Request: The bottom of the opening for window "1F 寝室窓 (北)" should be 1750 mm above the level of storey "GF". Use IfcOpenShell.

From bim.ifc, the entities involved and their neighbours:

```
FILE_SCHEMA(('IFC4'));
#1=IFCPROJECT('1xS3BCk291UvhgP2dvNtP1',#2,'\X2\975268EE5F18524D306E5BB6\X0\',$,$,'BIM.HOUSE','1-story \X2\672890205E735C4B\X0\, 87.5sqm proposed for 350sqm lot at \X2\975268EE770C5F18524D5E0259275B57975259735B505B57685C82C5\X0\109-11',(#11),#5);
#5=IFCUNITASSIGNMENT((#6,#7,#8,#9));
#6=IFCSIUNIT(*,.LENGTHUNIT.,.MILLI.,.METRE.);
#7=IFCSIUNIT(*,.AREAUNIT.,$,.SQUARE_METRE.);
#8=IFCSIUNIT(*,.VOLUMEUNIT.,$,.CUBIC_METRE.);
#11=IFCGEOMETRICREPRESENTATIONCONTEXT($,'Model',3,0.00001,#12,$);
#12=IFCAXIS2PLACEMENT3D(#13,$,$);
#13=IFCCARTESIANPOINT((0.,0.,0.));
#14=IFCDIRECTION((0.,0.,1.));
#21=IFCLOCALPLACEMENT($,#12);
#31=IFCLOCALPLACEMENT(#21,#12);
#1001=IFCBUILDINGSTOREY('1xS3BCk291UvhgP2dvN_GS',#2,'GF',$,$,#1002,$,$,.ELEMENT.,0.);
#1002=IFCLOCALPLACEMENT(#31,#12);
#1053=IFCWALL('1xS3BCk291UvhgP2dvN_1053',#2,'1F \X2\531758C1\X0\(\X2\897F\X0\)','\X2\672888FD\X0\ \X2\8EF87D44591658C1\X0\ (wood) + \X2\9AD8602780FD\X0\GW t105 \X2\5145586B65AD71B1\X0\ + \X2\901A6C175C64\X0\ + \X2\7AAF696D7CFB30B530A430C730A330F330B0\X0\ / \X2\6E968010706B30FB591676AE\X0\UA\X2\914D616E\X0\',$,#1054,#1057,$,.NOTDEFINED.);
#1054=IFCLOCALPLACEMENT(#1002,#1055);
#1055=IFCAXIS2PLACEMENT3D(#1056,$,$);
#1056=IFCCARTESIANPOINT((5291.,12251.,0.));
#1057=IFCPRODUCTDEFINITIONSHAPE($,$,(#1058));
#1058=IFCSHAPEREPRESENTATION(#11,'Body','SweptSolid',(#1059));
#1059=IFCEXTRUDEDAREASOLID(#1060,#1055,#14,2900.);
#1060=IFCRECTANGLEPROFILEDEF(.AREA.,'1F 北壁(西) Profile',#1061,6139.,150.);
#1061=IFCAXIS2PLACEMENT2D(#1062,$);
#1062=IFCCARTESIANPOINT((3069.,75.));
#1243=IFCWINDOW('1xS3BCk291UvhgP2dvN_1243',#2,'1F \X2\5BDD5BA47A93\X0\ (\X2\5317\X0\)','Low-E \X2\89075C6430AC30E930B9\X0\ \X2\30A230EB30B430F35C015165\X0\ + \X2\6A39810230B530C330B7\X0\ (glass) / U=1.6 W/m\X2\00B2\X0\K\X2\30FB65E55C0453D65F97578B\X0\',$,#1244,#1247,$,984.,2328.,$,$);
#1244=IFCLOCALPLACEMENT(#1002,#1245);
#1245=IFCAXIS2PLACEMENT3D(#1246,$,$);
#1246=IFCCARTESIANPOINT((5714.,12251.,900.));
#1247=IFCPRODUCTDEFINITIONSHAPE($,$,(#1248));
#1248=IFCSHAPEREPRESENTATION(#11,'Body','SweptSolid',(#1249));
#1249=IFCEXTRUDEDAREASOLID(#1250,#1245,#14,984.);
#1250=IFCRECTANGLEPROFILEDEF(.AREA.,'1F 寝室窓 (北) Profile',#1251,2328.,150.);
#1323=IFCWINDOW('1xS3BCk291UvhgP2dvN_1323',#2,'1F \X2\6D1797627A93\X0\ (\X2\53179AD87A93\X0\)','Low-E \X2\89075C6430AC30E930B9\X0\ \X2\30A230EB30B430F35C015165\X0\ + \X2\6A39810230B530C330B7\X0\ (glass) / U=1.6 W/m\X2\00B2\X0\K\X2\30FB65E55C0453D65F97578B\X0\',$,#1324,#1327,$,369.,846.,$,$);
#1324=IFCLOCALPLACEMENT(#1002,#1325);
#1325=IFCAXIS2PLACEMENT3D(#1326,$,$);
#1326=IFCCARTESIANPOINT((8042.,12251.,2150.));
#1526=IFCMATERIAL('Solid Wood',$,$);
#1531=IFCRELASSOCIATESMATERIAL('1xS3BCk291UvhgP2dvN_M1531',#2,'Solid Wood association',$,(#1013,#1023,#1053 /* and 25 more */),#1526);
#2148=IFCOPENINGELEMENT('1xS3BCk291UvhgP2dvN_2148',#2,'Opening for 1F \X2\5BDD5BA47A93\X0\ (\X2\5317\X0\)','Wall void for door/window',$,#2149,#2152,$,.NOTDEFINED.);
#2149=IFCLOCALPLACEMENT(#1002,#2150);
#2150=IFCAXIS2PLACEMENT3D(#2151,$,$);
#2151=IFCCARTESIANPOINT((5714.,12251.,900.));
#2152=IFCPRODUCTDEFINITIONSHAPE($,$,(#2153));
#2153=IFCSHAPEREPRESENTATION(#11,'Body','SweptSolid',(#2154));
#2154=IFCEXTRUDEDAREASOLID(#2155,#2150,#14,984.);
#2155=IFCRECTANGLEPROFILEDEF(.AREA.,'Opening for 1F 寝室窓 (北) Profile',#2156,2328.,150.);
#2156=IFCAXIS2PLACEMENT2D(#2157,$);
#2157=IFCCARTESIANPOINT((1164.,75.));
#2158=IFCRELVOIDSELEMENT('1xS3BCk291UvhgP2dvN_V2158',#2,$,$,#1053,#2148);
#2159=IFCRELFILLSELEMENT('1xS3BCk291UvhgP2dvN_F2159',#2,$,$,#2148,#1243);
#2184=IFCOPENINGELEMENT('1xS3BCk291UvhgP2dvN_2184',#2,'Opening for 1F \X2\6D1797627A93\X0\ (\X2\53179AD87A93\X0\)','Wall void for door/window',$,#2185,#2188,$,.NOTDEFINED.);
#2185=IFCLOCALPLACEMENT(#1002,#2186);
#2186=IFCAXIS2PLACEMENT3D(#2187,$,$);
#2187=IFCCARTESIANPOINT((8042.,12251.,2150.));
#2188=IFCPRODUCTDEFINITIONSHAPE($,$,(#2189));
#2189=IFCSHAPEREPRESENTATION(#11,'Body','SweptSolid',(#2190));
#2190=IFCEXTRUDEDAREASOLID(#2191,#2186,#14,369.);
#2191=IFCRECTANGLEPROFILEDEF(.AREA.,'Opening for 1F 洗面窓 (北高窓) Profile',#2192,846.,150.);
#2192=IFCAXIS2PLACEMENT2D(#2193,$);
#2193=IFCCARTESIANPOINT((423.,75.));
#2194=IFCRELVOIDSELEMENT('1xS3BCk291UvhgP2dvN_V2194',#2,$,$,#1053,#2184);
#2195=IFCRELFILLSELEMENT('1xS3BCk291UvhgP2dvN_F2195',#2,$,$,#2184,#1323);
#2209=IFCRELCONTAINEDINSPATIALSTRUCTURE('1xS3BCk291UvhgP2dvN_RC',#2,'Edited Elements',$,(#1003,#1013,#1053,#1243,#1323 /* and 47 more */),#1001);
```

```python
import numpy as np
import ifcopenshell
import ifcopenshell.api.geometry
import ifcopenshell.geom
import ifcopenshell.util.element
import ifcopenshell.util.placement
import ifcopenshell.util.shape
import ifcopenshell.util.unit

model = ifcopenshell.open("bim.ifc")
unit_scale = ifcopenshell.util.unit.calculate_unit_scale(model)

window = model.by_id(1243)
opening = window.FillsVoids[0].RelatingOpeningElement
storey = ifcopenshell.util.element.get_container(window, ifc_class="IfcBuildingStorey")
level = ifcopenshell.util.placement.get_local_placement(storey.ObjectPlacement)[2, 3]

# The opening's origin need not be at the sill, so measure its lowest point.
shape = ifcopenshell.geom.create_shape(ifcopenshell.geom.settings(), opening)
bottom = ifcopenshell.util.shape.get_shape_bottom_elevation(shape, shape.geometry) / unit_scale
dz = level + 1750.0 - bottom

shift = np.array([0.0, 0.0, dz])
# The window is not placed relative to its opening, so move both.
for product in (opening, window):
    matrix = ifcopenshell.util.placement.get_local_placement(product.ObjectPlacement)
    matrix[:3, 3] += shift
    ifcopenshell.api.geometry.edit_object_placement(model, product=product, matrix=matrix, is_si=False)

print(f"moved by {dz * unit_scale:+.3f} m")

model.write("bim_rev.ifc")
```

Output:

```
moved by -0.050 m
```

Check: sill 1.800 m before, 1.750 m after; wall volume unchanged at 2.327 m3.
